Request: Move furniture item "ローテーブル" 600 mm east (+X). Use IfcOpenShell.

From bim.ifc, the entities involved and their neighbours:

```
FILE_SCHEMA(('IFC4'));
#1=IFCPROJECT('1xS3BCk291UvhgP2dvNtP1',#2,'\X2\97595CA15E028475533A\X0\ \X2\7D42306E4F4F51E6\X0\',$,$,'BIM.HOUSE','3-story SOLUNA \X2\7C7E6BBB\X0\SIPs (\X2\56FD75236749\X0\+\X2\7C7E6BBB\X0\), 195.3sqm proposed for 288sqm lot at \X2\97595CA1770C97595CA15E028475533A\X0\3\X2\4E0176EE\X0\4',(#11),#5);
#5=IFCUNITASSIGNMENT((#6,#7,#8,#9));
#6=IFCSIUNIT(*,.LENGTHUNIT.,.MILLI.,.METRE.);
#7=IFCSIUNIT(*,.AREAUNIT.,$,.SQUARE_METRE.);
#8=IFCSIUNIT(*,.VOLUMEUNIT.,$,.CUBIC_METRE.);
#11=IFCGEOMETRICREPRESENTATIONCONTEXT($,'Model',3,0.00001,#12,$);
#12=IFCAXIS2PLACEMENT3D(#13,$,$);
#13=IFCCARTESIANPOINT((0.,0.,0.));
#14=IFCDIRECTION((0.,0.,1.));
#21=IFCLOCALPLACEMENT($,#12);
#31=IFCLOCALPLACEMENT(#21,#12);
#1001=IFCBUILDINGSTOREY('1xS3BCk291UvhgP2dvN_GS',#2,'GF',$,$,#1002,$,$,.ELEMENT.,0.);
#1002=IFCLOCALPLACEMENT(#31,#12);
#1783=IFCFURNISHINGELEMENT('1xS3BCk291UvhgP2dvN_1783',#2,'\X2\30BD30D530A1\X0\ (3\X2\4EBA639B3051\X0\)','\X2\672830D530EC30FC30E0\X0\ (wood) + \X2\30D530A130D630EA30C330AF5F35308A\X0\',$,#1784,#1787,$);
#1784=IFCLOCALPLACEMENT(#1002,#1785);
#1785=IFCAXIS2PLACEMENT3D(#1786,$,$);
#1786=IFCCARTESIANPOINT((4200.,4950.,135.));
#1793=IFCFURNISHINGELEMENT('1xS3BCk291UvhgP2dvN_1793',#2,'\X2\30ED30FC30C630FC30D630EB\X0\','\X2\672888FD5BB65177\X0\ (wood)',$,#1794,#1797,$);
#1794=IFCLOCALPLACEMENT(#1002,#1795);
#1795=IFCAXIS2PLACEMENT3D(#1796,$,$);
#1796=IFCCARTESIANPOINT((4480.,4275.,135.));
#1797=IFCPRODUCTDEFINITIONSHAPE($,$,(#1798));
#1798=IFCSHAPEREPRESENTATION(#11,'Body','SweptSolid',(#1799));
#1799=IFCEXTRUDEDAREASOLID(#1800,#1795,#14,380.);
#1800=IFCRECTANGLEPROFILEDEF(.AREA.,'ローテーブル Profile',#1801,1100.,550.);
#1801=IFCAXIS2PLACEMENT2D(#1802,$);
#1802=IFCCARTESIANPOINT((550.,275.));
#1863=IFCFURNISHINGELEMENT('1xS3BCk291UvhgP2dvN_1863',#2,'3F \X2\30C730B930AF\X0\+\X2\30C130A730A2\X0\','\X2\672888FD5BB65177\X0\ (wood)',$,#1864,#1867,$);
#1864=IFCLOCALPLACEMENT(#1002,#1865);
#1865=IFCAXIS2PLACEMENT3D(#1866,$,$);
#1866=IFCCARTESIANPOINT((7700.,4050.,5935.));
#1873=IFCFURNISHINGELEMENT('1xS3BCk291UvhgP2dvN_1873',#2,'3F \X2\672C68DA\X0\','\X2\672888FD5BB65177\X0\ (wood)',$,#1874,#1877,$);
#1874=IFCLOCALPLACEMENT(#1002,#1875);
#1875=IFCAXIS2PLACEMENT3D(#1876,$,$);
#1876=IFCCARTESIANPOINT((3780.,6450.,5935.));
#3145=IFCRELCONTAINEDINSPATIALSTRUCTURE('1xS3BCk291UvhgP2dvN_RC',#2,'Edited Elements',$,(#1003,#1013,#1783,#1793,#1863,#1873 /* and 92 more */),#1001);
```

```python
import ifcopenshell
import ifcopenshell.api.geometry
import ifcopenshell.util.placement

model = ifcopenshell.open("bim.ifc")

item = model.by_guid("1xS3BCk291UvhgP2dvN_1793")
matrix = ifcopenshell.util.placement.get_local_placement(item.ObjectPlacement)
matrix[0, 3] += 600.0
ifcopenshell.api.geometry.edit_object_placement(model, product=item, matrix=matrix, is_si=False)

print(ifcopenshell.util.placement.get_local_placement(item.ObjectPlacement).round(3) + 0.0)

model.write("bim_v2.ifc")
```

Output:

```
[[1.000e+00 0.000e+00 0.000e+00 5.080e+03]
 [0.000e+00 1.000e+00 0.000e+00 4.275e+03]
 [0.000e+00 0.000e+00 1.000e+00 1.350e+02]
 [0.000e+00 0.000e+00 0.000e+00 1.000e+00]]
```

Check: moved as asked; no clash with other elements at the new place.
